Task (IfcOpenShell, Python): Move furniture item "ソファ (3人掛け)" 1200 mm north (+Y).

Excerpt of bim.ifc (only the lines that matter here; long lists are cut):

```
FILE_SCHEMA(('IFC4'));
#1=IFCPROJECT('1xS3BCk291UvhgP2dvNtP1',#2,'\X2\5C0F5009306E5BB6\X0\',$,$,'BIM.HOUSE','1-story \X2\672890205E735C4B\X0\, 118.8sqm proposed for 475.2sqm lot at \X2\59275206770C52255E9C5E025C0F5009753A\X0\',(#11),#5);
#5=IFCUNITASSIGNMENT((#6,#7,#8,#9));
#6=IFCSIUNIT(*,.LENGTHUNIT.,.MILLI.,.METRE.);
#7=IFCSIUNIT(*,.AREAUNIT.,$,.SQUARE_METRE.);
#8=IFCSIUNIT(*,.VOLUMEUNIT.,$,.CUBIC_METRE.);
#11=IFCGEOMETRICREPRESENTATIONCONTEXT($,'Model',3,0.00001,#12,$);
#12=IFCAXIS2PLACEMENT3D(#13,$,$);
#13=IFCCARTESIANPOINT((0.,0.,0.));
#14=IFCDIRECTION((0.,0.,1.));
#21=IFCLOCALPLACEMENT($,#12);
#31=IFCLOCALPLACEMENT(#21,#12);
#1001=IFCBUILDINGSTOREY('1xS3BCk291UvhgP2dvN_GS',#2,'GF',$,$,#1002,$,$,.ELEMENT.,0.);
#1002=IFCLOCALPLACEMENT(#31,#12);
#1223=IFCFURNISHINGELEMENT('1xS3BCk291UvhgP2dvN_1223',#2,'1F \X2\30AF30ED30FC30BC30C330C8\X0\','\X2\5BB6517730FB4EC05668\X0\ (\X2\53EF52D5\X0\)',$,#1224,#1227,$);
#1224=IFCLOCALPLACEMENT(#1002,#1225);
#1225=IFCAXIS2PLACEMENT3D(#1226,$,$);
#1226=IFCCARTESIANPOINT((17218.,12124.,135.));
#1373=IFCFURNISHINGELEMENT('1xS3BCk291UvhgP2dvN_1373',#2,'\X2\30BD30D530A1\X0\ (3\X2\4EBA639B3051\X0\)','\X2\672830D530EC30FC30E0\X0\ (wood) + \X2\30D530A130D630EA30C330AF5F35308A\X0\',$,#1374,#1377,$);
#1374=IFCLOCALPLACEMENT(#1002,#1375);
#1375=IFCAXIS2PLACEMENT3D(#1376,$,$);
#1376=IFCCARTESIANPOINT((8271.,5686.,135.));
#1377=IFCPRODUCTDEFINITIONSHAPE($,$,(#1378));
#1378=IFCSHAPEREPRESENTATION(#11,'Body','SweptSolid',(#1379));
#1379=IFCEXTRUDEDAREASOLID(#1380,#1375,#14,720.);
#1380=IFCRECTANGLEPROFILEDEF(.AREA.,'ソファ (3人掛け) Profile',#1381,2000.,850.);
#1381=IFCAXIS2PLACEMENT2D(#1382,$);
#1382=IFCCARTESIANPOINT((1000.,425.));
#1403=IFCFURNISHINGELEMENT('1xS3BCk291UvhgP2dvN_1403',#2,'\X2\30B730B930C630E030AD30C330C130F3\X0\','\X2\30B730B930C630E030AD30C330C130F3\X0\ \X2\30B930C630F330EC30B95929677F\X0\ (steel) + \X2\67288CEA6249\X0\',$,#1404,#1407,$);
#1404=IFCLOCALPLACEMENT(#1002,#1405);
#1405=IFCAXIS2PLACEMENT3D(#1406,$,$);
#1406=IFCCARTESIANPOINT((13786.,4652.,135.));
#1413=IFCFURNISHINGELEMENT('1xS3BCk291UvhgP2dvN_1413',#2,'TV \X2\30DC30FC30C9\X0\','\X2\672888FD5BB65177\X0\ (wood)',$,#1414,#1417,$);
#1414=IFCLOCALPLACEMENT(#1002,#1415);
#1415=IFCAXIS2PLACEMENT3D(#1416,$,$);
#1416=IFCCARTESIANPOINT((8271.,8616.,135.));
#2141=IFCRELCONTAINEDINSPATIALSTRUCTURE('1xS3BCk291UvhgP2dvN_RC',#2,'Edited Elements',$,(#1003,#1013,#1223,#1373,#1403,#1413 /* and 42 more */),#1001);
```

```python
import ifcopenshell
import ifcopenshell.api.geometry
import ifcopenshell.util.placement
import ifcopenshell.util.unit

model = ifcopenshell.open("bim.ifc")
unit_scale = ifcopenshell.util.unit.calculate_unit_scale(model)

item = model.by_id(1373)
matrix = ifcopenshell.util.placement.get_local_placement(item.ObjectPlacement)
matrix[1, 3] += 1.2 / unit_scale
ifcopenshell.api.geometry.edit_object_placement(model, product=item, matrix=matrix, is_si=False)

print(ifcopenshell.util.placement.get_local_placement(item.ObjectPlacement).round(3) + 0.0)

model.write("bim_v2.ifc")
```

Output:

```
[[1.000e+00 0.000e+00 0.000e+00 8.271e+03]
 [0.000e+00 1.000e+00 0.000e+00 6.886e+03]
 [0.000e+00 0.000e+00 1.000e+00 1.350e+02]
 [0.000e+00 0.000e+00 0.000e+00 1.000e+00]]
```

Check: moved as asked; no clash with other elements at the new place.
